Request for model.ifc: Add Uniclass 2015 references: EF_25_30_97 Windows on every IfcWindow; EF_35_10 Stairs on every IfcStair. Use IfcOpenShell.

First a look at what the model holds.

```python
import ifcopenshell

model = ifcopenshell.open("model.ifc")
print(model.schema)
print("classifications:", [c.Name for c in model.by_type("IfcClassification")])
for ifc_class in ("IfcDoor", "IfcRoof", "IfcStair", "IfcWall", "IfcWindow"):
    print(ifc_class, len(model.by_type(ifc_class)))
```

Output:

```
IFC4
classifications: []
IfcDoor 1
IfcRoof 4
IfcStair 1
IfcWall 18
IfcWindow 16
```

```python
import ifcopenshell
import ifcopenshell.api.classification

model = ifcopenshell.open("model.ifc")

system = ifcopenshell.api.classification.add_classification(model, classification="Uniclass 2015")

codes = {
    "IfcWindow": ("EF_25_30_97", "Windows"),
    "IfcStair": ("EF_35_10", "Stairs"),
}
for ifc_class, (code, name) in codes.items():
    products = model.by_type(ifc_class)
    ifcopenshell.api.classification.add_reference(
        model, products=products, classification=system, identification=code, name=name
    )
    print(code, len(products))

model.write("model_edited.ifc")
```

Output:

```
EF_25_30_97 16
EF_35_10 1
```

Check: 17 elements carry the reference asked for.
